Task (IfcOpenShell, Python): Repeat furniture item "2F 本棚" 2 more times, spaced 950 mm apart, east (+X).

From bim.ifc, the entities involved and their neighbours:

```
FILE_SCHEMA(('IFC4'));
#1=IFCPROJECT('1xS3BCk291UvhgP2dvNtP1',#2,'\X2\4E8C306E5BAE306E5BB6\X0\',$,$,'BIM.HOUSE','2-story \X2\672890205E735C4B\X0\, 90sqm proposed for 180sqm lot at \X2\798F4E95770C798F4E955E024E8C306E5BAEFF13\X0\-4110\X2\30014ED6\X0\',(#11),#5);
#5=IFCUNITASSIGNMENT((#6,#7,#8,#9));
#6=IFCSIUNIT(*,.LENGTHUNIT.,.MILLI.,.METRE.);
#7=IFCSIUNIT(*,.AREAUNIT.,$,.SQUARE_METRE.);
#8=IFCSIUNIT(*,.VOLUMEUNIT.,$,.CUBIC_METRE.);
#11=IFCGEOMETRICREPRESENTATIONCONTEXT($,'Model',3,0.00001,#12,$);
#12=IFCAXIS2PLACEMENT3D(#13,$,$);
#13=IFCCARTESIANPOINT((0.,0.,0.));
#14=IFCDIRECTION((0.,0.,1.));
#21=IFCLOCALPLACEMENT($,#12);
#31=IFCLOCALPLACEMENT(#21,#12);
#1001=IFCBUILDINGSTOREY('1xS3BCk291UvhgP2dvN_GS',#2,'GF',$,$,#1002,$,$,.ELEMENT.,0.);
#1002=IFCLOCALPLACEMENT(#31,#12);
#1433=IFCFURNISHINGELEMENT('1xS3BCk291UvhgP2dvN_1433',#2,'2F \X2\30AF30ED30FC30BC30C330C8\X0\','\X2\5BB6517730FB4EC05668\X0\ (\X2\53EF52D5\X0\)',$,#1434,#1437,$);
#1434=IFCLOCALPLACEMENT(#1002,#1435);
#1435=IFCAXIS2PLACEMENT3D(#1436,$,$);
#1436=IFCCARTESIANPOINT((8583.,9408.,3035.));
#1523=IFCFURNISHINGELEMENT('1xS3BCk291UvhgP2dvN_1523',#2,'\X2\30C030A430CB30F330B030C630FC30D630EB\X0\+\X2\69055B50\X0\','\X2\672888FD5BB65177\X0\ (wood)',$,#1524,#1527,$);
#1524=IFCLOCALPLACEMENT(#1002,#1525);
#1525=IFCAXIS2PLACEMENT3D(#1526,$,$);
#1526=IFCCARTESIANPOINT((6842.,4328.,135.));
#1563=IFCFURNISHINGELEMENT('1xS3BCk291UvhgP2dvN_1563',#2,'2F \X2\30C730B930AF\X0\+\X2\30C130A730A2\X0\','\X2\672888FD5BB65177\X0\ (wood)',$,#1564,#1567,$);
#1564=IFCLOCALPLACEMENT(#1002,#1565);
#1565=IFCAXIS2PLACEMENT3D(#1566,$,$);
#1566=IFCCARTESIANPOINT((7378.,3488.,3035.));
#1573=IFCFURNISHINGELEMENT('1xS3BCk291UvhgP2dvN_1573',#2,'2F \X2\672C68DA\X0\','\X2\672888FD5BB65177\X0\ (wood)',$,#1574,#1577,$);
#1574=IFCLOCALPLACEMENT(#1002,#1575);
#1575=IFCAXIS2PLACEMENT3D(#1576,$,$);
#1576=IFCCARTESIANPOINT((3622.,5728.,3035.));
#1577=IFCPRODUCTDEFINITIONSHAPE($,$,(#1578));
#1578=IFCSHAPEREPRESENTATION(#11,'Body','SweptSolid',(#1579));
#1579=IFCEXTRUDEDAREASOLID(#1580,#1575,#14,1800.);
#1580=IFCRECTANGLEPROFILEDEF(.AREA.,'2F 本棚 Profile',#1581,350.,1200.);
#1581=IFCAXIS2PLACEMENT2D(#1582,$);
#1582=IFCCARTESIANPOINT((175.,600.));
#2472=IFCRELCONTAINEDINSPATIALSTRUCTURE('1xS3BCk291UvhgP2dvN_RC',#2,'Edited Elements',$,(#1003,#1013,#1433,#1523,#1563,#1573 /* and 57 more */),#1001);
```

```python
import numpy as np
import ifcopenshell
import ifcopenshell.api.geometry
import ifcopenshell.api.root
import ifcopenshell.util.element
import ifcopenshell.util.placement
import ifcopenshell.util.unit

model = ifcopenshell.open("bim.ifc")
unit_scale = ifcopenshell.util.unit.calculate_unit_scale(model)


def reuse_history(source, copy):
    """copy_class also copies each property set's owner history, people and application; keep the originals."""
    for rel in copy.IsDefinedBy:
        if rel.is_a("IfcRelDefinesByProperties") and (history := rel.RelatingPropertyDefinition.OwnerHistory):
            rel.RelatingPropertyDefinition.OwnerHistory = source.OwnerHistory
            ifcopenshell.util.element.remove_deep2(model, history)


source = model.by_id(1573)
base = ifcopenshell.util.placement.get_local_placement(source.ObjectPlacement)
step = np.array([1.0, 0.0, 0.0]) * 0.95 / unit_scale

for i in range(1, 3):
    copy = ifcopenshell.api.root.copy_class(model, product=source)
    copy.Representation = ifcopenshell.util.element.copy_deep(
        model, source.Representation, exclude=["IfcGeometricRepresentationContext", "IfcRepresentationMap"]
    )
    reuse_history(source, copy)
    matrix = base.copy()
    matrix[:3, 3] += i * step
    print("added at", matrix[:3, 3].round(3) + 0.0)
    ifcopenshell.api.geometry.edit_object_placement(model, product=copy, matrix=matrix, is_si=False)

model.write("bim-out.ifc")
```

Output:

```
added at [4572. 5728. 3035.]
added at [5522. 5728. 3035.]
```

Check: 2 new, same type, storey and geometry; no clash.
